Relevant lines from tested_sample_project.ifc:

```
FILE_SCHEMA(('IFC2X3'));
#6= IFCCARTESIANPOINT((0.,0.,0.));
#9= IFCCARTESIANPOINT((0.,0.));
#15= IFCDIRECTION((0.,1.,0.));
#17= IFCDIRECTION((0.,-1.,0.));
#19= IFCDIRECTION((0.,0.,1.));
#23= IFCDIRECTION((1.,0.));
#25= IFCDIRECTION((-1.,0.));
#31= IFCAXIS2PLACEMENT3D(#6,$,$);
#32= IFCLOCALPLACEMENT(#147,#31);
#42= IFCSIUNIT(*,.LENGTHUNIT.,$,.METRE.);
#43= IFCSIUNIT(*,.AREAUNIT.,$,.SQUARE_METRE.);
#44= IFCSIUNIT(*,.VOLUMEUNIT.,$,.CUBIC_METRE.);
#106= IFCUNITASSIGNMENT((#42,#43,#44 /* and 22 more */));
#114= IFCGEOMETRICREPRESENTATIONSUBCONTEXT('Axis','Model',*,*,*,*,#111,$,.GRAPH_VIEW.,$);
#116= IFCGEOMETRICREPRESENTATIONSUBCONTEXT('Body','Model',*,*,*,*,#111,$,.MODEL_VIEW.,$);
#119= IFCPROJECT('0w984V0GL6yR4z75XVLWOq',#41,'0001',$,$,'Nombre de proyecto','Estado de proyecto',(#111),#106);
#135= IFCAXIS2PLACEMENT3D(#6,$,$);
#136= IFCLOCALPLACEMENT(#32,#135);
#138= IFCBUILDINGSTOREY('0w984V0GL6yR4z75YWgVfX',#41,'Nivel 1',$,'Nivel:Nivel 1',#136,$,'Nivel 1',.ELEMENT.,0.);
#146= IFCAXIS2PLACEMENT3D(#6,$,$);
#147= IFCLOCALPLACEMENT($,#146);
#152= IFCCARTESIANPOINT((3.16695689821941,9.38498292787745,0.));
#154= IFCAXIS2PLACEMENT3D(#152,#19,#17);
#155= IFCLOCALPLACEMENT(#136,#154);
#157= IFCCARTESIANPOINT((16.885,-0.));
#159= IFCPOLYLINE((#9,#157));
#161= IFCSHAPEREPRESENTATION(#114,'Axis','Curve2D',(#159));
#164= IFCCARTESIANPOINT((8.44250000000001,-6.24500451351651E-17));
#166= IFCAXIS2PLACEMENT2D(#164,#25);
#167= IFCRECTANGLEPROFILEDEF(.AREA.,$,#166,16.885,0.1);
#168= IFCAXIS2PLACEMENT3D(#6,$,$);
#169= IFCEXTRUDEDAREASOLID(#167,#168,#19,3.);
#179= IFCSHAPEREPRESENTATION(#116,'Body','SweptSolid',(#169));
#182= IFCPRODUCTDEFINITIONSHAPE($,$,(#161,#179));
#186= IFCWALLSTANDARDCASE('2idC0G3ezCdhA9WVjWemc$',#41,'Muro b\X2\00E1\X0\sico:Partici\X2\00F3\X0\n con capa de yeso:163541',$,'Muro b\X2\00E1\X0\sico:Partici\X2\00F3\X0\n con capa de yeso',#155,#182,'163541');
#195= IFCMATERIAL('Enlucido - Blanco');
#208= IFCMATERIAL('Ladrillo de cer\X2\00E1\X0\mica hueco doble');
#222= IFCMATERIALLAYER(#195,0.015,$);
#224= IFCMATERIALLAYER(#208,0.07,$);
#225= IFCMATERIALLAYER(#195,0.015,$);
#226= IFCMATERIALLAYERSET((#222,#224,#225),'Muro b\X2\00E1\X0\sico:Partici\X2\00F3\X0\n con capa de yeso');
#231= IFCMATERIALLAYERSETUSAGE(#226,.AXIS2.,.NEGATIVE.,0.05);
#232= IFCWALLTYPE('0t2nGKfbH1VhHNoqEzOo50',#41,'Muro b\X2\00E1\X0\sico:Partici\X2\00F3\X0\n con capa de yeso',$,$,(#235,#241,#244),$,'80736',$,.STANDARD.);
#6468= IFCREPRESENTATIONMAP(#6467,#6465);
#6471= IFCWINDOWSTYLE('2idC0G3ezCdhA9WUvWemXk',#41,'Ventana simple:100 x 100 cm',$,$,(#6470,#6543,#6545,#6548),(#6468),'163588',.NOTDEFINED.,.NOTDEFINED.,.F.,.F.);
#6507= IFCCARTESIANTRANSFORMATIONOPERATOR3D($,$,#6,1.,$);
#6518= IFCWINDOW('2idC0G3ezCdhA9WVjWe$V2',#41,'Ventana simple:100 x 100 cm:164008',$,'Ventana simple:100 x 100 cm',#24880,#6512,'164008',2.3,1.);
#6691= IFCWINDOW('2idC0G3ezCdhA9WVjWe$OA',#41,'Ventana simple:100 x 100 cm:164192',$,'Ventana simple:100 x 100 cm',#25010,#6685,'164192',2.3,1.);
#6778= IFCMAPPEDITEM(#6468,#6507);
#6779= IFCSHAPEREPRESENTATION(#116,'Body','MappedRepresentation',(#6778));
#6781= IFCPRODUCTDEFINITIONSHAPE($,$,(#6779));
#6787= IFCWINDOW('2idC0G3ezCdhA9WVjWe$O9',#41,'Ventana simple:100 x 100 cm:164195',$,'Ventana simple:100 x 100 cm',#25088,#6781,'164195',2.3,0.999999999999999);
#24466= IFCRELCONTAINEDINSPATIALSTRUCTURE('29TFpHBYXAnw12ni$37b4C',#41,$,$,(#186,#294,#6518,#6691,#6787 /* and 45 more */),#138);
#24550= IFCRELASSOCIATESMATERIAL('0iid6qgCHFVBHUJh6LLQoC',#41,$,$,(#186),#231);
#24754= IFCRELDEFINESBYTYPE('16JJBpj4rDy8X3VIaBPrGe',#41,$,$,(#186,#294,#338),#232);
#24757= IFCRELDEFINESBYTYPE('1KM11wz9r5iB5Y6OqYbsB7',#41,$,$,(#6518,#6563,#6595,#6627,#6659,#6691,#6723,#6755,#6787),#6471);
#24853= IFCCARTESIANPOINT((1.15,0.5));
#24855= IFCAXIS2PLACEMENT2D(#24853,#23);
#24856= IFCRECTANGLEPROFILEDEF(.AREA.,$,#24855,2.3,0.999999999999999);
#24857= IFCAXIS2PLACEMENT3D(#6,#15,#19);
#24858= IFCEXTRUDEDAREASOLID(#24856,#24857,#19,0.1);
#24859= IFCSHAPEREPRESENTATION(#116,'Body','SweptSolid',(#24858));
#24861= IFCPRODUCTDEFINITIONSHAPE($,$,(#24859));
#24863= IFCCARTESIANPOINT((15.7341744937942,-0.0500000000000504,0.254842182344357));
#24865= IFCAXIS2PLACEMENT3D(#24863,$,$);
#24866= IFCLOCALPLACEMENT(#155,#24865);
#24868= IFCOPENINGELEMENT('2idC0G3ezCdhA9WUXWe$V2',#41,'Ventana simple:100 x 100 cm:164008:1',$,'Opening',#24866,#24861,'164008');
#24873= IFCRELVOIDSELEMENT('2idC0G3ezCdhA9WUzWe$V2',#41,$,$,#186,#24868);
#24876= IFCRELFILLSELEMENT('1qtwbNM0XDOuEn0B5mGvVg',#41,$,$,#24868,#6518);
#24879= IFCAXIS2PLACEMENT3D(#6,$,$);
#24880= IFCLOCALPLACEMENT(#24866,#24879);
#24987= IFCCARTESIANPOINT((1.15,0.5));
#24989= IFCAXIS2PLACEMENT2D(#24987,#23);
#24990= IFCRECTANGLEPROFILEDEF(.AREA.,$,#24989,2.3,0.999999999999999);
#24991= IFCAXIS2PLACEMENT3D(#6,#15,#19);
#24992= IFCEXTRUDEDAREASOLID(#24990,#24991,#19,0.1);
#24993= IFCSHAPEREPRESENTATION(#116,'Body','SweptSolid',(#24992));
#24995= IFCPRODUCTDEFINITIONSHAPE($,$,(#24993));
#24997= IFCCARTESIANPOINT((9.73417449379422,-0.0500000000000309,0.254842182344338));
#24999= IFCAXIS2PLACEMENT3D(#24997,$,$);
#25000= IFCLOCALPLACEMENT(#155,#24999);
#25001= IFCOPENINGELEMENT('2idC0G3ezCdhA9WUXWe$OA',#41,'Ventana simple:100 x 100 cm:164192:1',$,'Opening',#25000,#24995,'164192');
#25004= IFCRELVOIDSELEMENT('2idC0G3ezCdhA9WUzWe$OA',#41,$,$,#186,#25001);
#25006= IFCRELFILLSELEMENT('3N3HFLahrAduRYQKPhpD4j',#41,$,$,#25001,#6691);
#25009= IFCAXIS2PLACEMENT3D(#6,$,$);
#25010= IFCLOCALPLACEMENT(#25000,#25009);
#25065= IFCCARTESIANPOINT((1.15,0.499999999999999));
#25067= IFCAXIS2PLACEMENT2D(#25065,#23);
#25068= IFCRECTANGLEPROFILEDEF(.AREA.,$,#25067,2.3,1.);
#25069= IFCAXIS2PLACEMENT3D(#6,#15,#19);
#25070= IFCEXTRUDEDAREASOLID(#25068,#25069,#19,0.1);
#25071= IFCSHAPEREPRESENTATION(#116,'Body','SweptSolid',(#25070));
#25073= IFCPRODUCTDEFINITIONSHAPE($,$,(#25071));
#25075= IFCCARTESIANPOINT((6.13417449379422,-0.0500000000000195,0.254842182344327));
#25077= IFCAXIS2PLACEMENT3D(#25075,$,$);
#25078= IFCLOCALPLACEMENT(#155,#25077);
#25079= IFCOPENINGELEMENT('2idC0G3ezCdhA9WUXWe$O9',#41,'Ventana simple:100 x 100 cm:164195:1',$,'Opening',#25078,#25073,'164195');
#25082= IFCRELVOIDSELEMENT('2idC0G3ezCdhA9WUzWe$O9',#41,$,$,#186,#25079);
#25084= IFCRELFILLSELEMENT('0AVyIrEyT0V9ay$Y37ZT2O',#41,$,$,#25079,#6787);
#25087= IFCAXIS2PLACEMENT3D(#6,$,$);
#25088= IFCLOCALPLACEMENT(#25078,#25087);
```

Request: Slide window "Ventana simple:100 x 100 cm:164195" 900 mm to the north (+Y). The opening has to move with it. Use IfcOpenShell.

```python
import ifcopenshell
import ifcopenshell.api.geometry
import ifcopenshell.util.placement

model = ifcopenshell.open("tested_sample_project.ifc")

window = model.by_guid("2idC0G3ezCdhA9WVjWe$O9")
opening = window.FillsVoids[0].RelatingOpeningElement
wall = opening.VoidsElements[0].RelatingBuildingElement

wall_matrix = ifcopenshell.util.placement.get_local_placement(wall.ObjectPlacement)
shift = wall_matrix[:3, 0] * -0.9
before = ifcopenshell.util.placement.get_local_placement(window.ObjectPlacement)[:3, 3].copy()

# The window is placed relative to its opening, so it follows when the opening moves.
matrix = ifcopenshell.util.placement.get_local_placement(opening.ObjectPlacement)
matrix[:3, 3] += shift
ifcopenshell.api.geometry.edit_object_placement(
    model, product=opening, matrix=matrix, is_si=False, should_transform_children=True
)

after = ifcopenshell.util.placement.get_local_placement(window.ObjectPlacement)[:3, 3]
print("window moved by", (after - before).round(3) + 0.0)

model.write("tested_sample_project_rev.ifc")
```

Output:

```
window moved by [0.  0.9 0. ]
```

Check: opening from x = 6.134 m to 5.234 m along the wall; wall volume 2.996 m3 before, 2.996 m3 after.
